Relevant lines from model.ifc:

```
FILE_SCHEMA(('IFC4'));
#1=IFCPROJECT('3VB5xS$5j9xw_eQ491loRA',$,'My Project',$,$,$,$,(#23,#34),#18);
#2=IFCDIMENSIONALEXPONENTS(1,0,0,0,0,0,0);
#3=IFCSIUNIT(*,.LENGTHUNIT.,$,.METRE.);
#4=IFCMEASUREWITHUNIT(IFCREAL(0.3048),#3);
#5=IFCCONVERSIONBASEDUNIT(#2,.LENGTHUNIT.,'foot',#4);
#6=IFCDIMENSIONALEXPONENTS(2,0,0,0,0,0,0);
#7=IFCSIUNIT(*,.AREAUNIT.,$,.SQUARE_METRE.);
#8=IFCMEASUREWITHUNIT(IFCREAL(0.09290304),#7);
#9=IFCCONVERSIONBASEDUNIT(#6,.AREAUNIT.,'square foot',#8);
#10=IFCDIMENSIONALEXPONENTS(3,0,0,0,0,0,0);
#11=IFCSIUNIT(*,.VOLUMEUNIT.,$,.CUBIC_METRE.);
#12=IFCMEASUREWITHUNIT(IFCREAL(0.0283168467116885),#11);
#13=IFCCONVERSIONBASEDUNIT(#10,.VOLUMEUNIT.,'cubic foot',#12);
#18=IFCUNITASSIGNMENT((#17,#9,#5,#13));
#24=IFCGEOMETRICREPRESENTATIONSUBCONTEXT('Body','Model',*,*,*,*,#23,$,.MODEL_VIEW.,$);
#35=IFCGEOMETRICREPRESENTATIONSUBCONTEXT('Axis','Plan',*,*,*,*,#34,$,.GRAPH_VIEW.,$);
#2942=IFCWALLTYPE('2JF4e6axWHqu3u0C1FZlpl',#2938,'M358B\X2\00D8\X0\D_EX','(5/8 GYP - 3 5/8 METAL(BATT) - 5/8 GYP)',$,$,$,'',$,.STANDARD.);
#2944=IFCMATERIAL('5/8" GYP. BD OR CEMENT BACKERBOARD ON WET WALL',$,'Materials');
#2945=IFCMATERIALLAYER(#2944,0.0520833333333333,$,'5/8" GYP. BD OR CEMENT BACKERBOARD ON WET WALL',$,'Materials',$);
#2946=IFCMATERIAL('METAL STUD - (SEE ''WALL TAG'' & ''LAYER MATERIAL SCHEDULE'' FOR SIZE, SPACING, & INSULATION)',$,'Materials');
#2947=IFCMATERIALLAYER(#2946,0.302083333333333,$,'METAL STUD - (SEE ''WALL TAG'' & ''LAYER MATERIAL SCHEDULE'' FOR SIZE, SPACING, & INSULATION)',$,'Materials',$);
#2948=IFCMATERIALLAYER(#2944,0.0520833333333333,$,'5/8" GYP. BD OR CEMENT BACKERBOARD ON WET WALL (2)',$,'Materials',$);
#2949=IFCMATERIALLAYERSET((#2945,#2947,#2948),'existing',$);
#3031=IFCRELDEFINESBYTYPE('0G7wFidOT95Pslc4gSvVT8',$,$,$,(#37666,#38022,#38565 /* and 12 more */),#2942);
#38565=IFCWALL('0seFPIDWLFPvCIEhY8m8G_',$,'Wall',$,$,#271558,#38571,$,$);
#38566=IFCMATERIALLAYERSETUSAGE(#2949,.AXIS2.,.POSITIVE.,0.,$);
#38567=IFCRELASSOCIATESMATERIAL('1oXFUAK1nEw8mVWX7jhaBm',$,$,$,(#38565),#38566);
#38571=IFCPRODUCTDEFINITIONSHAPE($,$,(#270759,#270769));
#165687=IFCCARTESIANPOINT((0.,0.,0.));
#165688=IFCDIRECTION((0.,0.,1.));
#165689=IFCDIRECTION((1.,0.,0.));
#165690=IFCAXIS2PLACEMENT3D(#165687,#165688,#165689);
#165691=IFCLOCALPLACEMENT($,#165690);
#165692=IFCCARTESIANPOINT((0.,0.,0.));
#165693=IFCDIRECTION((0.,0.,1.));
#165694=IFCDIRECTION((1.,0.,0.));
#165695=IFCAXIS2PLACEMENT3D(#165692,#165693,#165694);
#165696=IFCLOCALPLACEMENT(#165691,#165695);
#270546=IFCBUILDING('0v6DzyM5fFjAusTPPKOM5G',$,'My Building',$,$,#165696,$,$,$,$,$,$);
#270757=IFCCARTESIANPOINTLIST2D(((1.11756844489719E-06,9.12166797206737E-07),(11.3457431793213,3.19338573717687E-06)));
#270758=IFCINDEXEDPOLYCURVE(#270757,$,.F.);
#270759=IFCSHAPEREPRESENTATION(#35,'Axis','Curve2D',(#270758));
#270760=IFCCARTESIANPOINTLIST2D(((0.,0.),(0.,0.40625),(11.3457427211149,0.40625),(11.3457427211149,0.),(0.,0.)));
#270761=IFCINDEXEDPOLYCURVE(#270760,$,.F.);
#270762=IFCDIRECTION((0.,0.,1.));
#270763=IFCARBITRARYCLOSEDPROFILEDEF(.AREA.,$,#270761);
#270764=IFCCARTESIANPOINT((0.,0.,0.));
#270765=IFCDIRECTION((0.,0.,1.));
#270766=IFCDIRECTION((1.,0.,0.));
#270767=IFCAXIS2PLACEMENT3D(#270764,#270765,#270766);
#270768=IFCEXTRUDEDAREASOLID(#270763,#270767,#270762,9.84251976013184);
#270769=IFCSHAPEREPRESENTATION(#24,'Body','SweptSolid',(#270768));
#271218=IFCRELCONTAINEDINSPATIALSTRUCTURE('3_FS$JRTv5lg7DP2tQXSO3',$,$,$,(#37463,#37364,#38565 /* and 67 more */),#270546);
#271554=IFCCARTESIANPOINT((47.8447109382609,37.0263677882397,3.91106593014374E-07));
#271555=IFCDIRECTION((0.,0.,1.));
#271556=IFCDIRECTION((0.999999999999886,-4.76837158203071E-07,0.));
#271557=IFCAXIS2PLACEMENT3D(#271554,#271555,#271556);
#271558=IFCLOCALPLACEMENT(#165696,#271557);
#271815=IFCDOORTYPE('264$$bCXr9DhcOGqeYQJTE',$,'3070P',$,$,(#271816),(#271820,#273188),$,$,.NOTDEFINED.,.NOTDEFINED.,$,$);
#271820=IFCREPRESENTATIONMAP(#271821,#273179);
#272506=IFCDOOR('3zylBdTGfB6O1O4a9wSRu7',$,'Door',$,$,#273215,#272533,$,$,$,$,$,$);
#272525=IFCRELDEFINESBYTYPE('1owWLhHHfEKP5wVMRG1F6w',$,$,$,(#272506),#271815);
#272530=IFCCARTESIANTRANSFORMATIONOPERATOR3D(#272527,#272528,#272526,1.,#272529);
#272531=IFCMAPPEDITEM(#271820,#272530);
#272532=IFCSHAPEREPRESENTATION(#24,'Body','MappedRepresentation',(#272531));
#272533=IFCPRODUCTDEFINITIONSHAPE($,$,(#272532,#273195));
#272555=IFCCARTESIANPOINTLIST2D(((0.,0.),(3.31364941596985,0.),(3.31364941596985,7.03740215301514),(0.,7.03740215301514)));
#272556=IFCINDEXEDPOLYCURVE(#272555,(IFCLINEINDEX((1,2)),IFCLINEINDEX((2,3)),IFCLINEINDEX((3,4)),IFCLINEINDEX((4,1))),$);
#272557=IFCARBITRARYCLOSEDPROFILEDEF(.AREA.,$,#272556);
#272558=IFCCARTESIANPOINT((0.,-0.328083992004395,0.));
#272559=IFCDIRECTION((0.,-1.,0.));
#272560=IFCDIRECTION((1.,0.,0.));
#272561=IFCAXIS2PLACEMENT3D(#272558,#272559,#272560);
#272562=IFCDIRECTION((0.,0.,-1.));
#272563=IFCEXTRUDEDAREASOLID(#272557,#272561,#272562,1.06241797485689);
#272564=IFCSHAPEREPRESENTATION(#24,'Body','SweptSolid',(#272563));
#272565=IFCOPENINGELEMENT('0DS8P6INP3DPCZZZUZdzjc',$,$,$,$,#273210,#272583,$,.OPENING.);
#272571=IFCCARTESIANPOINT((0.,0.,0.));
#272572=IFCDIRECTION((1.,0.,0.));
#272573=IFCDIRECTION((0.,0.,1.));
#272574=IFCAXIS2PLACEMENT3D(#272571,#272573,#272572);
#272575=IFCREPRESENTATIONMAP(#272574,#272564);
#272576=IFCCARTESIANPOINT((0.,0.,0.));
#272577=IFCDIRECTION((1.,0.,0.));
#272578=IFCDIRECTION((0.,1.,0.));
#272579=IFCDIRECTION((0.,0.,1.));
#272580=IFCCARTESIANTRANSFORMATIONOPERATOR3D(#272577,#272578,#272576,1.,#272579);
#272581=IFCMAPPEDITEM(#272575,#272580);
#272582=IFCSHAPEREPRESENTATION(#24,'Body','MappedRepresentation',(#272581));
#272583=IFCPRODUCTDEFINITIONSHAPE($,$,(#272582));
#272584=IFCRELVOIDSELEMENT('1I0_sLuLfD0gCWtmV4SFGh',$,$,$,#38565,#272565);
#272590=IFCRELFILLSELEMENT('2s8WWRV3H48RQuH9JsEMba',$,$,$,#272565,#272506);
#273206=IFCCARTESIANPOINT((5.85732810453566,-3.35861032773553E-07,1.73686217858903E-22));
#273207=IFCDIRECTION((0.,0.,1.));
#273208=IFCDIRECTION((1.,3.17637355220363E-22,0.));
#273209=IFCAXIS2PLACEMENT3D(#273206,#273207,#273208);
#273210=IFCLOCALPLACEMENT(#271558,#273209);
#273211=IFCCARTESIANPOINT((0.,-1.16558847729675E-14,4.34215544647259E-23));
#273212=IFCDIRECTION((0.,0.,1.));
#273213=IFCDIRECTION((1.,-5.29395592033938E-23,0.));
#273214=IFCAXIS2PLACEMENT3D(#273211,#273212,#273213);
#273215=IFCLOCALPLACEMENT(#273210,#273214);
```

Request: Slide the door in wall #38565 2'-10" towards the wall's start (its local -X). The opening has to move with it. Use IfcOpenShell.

```python
import ifcopenshell
import ifcopenshell.api.geometry
import ifcopenshell.util.placement
import ifcopenshell.util.unit

model = ifcopenshell.open("model.ifc")
unit_scale = ifcopenshell.util.unit.calculate_unit_scale(model)

door = model.by_guid("3zylBdTGfB6O1O4a9wSRu7")
opening = door.FillsVoids[0].RelatingOpeningElement
wall = opening.VoidsElements[0].RelatingBuildingElement

wall_matrix = ifcopenshell.util.placement.get_local_placement(wall.ObjectPlacement)
shift = wall_matrix[:3, 0] * -34 * 0.0254 / unit_scale
before = ifcopenshell.util.placement.get_local_placement(door.ObjectPlacement)[:3, 3].copy()

# The door is placed relative to its opening, so it follows when the opening moves.
matrix = ifcopenshell.util.placement.get_local_placement(opening.ObjectPlacement)
matrix[:3, 3] += shift
ifcopenshell.api.geometry.edit_object_placement(
    model, product=opening, matrix=matrix, is_si=False, should_transform_children=True
)

after = ifcopenshell.util.placement.get_local_placement(door.ObjectPlacement)[:3, 3]
print("door moved by", (after - before).round(3) + 0.0)

model.write("model_v2.ifc")
```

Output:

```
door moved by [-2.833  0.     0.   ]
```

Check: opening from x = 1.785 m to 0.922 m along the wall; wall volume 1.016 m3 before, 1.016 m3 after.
